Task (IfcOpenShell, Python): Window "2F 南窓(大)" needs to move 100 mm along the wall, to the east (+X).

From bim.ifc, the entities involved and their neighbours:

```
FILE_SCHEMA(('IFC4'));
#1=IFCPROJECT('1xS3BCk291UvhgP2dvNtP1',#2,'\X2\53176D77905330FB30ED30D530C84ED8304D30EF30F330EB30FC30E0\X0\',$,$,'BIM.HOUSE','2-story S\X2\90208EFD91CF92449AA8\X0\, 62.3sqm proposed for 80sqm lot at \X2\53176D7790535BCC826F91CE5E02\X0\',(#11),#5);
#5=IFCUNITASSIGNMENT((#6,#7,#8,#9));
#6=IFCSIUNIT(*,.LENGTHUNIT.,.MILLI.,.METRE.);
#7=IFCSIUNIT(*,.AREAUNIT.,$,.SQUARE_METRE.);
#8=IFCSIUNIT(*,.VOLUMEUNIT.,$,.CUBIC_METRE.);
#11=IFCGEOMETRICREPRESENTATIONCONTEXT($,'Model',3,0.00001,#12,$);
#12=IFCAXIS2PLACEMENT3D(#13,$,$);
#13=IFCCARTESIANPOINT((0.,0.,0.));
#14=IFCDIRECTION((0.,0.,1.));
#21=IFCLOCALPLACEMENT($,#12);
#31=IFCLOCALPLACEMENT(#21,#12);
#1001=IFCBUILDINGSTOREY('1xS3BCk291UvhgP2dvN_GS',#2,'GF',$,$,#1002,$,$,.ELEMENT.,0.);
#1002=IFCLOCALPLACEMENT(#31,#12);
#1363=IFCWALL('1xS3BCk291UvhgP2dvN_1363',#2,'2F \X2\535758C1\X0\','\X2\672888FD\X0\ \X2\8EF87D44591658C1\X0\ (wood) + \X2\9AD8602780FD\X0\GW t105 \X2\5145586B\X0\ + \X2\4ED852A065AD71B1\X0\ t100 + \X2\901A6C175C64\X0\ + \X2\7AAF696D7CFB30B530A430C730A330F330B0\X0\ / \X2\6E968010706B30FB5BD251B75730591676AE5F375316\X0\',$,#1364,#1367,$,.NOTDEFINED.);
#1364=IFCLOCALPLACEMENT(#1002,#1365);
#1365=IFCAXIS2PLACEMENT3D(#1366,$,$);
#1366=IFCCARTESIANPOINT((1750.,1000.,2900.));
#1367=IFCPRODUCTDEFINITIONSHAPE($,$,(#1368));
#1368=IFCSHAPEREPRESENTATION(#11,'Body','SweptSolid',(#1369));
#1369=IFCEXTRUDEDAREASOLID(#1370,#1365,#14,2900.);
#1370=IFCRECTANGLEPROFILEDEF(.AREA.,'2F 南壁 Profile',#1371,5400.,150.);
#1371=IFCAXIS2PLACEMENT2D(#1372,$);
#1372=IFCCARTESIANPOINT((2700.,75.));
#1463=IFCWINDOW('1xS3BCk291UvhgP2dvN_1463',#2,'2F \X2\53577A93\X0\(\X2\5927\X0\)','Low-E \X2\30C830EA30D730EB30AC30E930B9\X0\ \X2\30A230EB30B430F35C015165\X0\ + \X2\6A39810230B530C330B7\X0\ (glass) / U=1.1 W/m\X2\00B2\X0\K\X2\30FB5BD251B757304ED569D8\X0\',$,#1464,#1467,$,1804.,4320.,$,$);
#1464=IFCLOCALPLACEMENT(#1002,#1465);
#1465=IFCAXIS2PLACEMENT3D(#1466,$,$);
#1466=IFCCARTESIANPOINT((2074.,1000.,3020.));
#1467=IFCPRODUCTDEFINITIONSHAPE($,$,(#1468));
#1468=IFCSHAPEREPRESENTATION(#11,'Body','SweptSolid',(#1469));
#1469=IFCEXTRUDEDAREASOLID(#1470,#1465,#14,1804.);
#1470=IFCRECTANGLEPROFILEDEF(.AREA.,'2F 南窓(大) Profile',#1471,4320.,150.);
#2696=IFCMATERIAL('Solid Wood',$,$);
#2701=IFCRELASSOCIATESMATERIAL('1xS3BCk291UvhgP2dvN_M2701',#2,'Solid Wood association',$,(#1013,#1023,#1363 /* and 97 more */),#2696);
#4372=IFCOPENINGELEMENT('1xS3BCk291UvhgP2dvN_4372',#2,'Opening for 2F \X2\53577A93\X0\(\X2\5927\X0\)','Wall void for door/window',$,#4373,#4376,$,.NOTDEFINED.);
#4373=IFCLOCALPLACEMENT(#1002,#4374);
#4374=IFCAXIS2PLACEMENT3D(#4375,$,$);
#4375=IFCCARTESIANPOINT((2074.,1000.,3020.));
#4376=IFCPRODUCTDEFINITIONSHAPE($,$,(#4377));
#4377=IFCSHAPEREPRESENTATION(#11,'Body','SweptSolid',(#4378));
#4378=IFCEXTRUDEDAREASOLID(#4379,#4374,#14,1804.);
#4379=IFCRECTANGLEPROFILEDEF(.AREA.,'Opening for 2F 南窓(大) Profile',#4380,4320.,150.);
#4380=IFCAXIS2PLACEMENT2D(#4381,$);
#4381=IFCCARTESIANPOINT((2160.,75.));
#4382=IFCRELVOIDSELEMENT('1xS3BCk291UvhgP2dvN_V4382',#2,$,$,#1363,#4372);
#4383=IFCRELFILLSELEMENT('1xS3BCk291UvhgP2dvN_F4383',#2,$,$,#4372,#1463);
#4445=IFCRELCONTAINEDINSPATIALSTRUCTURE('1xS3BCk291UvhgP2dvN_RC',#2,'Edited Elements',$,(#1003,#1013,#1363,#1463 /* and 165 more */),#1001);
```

```python
import ifcopenshell
import ifcopenshell.api.geometry
import ifcopenshell.util.placement

model = ifcopenshell.open("bim.ifc")

window = model.by_guid("1xS3BCk291UvhgP2dvN_1463")
opening = window.FillsVoids[0].RelatingOpeningElement
wall = opening.VoidsElements[0].RelatingBuildingElement

wall_matrix = ifcopenshell.util.placement.get_local_placement(wall.ObjectPlacement)
shift = wall_matrix[:3, 0] * 100.0
before = ifcopenshell.util.placement.get_local_placement(window.ObjectPlacement)[:3, 3].copy()

# The window is not placed relative to its opening, so move both.
for product in (opening, window):
    matrix = ifcopenshell.util.placement.get_local_placement(product.ObjectPlacement)
    matrix[:3, 3] += shift
    ifcopenshell.api.geometry.edit_object_placement(model, product=product, matrix=matrix, is_si=False)

after = ifcopenshell.util.placement.get_local_placement(window.ObjectPlacement)[:3, 3]
print("window moved by", (after - before).round(3) + 0.0)

model.write("bim_edited.ifc")
```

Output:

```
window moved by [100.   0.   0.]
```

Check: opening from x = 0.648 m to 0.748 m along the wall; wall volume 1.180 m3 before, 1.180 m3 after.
